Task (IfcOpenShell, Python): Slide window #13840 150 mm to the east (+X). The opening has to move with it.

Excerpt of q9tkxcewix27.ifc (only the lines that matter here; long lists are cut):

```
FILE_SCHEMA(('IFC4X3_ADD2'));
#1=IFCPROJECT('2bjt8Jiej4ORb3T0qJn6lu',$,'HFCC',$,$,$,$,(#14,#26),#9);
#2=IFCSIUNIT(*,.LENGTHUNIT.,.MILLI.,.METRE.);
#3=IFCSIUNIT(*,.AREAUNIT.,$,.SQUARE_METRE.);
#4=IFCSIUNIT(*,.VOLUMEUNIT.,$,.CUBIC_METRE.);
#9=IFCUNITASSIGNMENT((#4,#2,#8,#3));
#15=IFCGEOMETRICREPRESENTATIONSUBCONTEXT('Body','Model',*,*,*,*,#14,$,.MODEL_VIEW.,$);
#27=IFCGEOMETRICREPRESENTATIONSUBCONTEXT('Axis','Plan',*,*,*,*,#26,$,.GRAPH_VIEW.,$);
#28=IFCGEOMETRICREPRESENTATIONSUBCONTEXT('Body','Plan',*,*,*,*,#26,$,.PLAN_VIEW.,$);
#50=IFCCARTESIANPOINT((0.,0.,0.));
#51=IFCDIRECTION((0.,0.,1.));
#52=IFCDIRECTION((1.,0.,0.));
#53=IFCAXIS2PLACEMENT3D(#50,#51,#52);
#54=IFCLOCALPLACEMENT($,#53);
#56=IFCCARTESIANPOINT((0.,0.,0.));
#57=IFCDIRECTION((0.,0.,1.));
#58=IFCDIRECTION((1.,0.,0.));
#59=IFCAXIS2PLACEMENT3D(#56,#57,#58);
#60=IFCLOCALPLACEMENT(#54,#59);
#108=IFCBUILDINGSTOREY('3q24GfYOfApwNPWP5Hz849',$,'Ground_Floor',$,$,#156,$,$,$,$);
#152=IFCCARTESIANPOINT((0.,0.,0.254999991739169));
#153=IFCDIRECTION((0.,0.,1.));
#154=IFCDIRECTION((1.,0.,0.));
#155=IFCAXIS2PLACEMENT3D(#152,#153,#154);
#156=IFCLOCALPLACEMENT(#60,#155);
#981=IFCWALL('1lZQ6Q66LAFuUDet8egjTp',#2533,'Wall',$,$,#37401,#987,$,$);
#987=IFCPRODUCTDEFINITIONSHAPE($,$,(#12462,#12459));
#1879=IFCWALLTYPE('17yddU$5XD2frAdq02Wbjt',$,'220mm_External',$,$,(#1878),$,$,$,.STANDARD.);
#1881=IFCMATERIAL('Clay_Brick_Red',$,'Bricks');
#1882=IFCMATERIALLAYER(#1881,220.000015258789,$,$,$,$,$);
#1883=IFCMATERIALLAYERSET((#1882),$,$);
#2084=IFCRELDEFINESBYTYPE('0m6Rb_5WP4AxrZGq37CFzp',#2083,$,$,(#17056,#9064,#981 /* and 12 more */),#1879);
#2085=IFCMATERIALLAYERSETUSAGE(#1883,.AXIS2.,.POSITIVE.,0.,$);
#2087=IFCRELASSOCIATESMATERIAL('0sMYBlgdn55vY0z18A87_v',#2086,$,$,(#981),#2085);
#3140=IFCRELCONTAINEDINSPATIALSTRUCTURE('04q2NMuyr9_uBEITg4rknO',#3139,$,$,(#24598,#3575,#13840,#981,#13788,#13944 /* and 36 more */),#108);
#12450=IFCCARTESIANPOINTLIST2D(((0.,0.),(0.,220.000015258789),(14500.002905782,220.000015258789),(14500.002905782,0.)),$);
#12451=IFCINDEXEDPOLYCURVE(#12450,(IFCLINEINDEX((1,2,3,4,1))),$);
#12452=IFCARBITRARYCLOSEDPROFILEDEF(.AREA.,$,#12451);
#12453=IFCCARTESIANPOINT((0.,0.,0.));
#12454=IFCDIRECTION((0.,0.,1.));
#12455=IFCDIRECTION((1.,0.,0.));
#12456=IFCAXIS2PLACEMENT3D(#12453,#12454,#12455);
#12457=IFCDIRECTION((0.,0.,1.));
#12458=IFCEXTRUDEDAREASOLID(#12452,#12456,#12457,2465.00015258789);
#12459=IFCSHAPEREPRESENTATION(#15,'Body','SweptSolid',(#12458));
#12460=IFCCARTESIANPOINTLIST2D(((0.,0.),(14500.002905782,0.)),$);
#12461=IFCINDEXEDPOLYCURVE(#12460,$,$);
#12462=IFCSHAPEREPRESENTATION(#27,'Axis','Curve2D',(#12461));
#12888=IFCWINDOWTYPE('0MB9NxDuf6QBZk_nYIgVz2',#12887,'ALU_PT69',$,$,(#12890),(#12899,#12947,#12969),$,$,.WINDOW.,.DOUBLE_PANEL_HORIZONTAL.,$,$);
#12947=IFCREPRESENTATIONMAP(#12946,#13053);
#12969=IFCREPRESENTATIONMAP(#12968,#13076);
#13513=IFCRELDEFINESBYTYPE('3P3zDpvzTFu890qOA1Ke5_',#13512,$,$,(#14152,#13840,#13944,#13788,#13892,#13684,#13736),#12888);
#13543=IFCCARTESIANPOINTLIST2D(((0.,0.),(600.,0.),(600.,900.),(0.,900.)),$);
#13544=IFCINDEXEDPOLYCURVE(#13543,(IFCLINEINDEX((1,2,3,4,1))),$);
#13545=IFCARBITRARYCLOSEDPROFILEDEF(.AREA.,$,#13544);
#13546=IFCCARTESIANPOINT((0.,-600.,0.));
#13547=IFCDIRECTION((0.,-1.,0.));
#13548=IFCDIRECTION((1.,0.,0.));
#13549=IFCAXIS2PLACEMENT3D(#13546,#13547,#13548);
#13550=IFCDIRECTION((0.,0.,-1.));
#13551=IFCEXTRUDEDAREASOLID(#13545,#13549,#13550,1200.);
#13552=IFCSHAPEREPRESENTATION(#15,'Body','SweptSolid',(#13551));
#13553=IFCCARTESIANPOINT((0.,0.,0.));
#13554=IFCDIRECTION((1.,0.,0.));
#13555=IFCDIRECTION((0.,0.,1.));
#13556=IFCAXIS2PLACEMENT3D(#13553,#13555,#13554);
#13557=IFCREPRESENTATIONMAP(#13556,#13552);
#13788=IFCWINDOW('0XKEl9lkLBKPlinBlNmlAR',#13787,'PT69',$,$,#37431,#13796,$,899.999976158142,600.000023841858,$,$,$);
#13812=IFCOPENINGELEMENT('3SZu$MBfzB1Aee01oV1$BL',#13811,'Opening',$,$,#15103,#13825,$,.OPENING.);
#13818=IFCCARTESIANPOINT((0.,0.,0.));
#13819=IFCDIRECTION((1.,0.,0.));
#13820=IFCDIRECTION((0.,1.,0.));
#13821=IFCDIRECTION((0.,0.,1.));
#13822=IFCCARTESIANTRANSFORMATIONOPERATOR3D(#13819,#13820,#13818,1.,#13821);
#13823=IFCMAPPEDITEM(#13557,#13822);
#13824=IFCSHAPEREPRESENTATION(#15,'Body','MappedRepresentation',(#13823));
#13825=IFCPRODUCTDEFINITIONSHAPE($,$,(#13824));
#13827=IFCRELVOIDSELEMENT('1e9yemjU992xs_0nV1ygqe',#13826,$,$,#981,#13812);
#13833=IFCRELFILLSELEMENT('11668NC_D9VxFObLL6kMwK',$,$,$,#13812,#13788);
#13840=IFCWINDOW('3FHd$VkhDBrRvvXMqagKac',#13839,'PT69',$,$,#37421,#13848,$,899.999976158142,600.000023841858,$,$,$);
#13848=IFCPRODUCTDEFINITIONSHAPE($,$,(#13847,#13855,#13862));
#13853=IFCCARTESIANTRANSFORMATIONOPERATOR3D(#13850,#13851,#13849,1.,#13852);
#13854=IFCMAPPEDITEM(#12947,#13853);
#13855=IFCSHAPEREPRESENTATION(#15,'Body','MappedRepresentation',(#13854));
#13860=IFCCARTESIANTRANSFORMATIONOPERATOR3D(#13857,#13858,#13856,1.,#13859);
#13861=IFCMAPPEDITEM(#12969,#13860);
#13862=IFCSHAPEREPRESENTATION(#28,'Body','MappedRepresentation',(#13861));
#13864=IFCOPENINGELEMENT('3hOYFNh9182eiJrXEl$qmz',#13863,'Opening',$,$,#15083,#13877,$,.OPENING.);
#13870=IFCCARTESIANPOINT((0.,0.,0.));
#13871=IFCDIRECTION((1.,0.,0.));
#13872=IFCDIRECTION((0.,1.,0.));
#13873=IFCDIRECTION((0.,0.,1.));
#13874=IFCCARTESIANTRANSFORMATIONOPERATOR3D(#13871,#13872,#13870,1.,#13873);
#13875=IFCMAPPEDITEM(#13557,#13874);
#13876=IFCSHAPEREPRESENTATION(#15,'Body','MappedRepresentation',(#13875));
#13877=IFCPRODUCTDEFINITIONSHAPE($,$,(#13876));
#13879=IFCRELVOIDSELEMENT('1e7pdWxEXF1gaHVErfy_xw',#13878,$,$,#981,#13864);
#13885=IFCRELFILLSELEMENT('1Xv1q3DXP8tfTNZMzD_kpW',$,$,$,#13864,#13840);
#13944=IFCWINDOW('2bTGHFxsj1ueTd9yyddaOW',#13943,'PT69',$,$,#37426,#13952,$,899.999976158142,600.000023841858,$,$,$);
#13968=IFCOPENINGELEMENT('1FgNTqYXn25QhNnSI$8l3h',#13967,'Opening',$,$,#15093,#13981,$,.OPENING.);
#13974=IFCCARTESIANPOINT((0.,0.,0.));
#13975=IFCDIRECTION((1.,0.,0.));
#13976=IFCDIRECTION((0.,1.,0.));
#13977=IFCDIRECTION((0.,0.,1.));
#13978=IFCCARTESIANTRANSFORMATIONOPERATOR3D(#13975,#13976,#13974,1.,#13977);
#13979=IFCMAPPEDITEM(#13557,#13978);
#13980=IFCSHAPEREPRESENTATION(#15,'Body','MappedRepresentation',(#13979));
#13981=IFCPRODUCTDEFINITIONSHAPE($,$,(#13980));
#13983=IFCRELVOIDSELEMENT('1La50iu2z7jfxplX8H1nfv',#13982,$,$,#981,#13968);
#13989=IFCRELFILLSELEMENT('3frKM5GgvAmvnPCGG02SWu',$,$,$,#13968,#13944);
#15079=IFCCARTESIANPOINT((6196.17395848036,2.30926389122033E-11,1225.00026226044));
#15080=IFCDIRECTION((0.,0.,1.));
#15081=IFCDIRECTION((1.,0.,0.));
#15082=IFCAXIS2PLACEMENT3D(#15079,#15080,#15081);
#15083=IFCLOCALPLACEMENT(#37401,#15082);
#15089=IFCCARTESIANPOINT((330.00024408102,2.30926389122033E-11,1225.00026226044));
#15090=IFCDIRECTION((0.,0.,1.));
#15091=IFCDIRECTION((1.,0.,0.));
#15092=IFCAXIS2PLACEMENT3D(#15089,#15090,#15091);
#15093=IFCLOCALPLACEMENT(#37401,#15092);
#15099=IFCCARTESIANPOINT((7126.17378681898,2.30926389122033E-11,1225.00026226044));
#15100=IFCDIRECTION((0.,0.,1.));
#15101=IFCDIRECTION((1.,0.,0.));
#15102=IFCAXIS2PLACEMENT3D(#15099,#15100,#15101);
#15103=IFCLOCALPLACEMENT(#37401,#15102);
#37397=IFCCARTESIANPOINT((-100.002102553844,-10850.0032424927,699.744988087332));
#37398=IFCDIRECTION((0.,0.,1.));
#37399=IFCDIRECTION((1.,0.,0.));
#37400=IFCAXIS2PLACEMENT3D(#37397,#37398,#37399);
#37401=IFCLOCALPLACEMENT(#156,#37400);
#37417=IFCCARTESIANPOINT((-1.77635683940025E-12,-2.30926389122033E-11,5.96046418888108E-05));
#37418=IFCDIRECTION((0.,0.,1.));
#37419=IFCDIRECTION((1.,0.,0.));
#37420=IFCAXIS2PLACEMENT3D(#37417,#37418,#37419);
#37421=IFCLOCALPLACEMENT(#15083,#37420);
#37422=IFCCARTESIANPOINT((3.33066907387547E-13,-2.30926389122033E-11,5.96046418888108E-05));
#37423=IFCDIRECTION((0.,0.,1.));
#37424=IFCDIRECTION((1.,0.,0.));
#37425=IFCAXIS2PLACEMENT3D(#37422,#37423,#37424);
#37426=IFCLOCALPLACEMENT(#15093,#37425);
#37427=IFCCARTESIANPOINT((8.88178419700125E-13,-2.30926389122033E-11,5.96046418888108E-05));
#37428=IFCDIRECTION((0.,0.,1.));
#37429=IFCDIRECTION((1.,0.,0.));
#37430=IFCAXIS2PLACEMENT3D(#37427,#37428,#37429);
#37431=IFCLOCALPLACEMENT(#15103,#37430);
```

```python
import ifcopenshell
import ifcopenshell.api.geometry
import ifcopenshell.util.placement
import ifcopenshell.util.unit

model = ifcopenshell.open("q9tkxcewix27.ifc")
unit_scale = ifcopenshell.util.unit.calculate_unit_scale(model)

window = model.by_guid("3FHd$VkhDBrRvvXMqagKac")
opening = window.FillsVoids[0].RelatingOpeningElement
wall = opening.VoidsElements[0].RelatingBuildingElement

wall_matrix = ifcopenshell.util.placement.get_local_placement(wall.ObjectPlacement)
shift = wall_matrix[:3, 0] * 0.15 / unit_scale
before = ifcopenshell.util.placement.get_local_placement(window.ObjectPlacement)[:3, 3].copy()

# The window is placed relative to its opening, so it follows when the opening moves.
matrix = ifcopenshell.util.placement.get_local_placement(opening.ObjectPlacement)
matrix[:3, 3] += shift
ifcopenshell.api.geometry.edit_object_placement(
    model, product=opening, matrix=matrix, is_si=False, should_transform_children=True
)

after = ifcopenshell.util.placement.get_local_placement(window.ObjectPlacement)[:3, 3]
print("window moved by", (after - before).round(3) + 0.0)

model.write("q9tkxcewix27_edited.ifc")
```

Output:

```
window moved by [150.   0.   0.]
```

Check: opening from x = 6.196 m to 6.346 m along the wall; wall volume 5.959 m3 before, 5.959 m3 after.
